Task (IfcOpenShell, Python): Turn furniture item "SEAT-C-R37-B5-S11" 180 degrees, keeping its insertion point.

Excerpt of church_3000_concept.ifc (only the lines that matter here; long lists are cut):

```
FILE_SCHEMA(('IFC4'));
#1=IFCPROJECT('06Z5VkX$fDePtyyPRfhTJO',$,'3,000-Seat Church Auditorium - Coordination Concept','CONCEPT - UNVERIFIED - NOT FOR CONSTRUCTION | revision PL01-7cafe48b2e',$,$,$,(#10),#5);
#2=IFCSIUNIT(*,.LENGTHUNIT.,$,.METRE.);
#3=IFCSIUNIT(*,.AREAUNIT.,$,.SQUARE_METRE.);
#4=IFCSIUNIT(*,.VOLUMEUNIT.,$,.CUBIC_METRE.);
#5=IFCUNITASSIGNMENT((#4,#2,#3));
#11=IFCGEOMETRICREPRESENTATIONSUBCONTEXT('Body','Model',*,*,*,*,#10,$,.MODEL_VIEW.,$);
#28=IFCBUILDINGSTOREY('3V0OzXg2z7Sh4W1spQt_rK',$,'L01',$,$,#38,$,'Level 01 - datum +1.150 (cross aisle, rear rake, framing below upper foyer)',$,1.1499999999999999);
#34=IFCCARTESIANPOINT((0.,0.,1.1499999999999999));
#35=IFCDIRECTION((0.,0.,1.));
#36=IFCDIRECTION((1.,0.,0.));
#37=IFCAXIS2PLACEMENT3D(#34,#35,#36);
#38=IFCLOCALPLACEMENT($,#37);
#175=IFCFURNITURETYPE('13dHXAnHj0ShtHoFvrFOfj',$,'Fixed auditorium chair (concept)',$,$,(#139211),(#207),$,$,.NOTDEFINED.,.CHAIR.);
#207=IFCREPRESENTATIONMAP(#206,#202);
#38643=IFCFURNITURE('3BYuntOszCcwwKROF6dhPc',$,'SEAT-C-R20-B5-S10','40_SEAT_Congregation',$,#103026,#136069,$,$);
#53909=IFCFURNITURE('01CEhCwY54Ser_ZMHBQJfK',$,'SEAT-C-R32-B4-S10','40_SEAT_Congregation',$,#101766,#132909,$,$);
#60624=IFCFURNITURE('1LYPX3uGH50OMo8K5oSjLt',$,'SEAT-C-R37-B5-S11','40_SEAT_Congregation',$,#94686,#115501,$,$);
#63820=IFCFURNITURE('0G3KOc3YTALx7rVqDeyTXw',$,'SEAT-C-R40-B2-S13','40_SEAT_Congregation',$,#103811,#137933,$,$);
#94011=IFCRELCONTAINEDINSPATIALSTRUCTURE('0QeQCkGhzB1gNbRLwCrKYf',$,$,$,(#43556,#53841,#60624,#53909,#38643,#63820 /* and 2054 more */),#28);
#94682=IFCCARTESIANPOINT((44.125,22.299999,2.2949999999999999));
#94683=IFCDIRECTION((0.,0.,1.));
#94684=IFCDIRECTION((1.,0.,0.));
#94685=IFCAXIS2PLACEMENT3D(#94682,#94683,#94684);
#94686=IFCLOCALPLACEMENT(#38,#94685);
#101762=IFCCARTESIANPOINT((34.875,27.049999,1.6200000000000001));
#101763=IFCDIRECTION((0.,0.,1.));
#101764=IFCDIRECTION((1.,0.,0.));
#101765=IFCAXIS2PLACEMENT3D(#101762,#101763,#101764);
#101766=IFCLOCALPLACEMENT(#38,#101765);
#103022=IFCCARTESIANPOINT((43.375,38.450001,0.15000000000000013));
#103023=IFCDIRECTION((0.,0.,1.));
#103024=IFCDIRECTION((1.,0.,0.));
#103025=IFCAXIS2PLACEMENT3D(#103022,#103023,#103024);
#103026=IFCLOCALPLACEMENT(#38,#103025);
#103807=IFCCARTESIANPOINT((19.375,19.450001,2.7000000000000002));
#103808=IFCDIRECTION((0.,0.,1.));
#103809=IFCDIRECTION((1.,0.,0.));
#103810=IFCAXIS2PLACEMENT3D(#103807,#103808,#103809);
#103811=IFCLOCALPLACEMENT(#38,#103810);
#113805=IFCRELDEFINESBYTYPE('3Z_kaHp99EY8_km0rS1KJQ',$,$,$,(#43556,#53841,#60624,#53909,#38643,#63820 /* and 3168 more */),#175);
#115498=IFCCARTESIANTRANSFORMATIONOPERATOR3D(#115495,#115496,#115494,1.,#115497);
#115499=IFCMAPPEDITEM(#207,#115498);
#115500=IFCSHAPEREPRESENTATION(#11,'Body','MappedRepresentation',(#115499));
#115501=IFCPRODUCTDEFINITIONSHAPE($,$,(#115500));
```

```python
import ifcopenshell
import ifcopenshell.api.geometry
import ifcopenshell.util.placement

model = ifcopenshell.open("church_3000_concept.ifc")

item = model.by_id(60624)
matrix = ifcopenshell.util.placement.get_local_placement(item.ObjectPlacement)
matrix = matrix @ ifcopenshell.util.placement.rotation(180, "Z")
ifcopenshell.api.geometry.edit_object_placement(model, product=item, matrix=matrix, is_si=False)

print(ifcopenshell.util.placement.get_local_placement(item.ObjectPlacement).round(3) + 0.0)

model.write("church_3000_concept_updated.ifc")
```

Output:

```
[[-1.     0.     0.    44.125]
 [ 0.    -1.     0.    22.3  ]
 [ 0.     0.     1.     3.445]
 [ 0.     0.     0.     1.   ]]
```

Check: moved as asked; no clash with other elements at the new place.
